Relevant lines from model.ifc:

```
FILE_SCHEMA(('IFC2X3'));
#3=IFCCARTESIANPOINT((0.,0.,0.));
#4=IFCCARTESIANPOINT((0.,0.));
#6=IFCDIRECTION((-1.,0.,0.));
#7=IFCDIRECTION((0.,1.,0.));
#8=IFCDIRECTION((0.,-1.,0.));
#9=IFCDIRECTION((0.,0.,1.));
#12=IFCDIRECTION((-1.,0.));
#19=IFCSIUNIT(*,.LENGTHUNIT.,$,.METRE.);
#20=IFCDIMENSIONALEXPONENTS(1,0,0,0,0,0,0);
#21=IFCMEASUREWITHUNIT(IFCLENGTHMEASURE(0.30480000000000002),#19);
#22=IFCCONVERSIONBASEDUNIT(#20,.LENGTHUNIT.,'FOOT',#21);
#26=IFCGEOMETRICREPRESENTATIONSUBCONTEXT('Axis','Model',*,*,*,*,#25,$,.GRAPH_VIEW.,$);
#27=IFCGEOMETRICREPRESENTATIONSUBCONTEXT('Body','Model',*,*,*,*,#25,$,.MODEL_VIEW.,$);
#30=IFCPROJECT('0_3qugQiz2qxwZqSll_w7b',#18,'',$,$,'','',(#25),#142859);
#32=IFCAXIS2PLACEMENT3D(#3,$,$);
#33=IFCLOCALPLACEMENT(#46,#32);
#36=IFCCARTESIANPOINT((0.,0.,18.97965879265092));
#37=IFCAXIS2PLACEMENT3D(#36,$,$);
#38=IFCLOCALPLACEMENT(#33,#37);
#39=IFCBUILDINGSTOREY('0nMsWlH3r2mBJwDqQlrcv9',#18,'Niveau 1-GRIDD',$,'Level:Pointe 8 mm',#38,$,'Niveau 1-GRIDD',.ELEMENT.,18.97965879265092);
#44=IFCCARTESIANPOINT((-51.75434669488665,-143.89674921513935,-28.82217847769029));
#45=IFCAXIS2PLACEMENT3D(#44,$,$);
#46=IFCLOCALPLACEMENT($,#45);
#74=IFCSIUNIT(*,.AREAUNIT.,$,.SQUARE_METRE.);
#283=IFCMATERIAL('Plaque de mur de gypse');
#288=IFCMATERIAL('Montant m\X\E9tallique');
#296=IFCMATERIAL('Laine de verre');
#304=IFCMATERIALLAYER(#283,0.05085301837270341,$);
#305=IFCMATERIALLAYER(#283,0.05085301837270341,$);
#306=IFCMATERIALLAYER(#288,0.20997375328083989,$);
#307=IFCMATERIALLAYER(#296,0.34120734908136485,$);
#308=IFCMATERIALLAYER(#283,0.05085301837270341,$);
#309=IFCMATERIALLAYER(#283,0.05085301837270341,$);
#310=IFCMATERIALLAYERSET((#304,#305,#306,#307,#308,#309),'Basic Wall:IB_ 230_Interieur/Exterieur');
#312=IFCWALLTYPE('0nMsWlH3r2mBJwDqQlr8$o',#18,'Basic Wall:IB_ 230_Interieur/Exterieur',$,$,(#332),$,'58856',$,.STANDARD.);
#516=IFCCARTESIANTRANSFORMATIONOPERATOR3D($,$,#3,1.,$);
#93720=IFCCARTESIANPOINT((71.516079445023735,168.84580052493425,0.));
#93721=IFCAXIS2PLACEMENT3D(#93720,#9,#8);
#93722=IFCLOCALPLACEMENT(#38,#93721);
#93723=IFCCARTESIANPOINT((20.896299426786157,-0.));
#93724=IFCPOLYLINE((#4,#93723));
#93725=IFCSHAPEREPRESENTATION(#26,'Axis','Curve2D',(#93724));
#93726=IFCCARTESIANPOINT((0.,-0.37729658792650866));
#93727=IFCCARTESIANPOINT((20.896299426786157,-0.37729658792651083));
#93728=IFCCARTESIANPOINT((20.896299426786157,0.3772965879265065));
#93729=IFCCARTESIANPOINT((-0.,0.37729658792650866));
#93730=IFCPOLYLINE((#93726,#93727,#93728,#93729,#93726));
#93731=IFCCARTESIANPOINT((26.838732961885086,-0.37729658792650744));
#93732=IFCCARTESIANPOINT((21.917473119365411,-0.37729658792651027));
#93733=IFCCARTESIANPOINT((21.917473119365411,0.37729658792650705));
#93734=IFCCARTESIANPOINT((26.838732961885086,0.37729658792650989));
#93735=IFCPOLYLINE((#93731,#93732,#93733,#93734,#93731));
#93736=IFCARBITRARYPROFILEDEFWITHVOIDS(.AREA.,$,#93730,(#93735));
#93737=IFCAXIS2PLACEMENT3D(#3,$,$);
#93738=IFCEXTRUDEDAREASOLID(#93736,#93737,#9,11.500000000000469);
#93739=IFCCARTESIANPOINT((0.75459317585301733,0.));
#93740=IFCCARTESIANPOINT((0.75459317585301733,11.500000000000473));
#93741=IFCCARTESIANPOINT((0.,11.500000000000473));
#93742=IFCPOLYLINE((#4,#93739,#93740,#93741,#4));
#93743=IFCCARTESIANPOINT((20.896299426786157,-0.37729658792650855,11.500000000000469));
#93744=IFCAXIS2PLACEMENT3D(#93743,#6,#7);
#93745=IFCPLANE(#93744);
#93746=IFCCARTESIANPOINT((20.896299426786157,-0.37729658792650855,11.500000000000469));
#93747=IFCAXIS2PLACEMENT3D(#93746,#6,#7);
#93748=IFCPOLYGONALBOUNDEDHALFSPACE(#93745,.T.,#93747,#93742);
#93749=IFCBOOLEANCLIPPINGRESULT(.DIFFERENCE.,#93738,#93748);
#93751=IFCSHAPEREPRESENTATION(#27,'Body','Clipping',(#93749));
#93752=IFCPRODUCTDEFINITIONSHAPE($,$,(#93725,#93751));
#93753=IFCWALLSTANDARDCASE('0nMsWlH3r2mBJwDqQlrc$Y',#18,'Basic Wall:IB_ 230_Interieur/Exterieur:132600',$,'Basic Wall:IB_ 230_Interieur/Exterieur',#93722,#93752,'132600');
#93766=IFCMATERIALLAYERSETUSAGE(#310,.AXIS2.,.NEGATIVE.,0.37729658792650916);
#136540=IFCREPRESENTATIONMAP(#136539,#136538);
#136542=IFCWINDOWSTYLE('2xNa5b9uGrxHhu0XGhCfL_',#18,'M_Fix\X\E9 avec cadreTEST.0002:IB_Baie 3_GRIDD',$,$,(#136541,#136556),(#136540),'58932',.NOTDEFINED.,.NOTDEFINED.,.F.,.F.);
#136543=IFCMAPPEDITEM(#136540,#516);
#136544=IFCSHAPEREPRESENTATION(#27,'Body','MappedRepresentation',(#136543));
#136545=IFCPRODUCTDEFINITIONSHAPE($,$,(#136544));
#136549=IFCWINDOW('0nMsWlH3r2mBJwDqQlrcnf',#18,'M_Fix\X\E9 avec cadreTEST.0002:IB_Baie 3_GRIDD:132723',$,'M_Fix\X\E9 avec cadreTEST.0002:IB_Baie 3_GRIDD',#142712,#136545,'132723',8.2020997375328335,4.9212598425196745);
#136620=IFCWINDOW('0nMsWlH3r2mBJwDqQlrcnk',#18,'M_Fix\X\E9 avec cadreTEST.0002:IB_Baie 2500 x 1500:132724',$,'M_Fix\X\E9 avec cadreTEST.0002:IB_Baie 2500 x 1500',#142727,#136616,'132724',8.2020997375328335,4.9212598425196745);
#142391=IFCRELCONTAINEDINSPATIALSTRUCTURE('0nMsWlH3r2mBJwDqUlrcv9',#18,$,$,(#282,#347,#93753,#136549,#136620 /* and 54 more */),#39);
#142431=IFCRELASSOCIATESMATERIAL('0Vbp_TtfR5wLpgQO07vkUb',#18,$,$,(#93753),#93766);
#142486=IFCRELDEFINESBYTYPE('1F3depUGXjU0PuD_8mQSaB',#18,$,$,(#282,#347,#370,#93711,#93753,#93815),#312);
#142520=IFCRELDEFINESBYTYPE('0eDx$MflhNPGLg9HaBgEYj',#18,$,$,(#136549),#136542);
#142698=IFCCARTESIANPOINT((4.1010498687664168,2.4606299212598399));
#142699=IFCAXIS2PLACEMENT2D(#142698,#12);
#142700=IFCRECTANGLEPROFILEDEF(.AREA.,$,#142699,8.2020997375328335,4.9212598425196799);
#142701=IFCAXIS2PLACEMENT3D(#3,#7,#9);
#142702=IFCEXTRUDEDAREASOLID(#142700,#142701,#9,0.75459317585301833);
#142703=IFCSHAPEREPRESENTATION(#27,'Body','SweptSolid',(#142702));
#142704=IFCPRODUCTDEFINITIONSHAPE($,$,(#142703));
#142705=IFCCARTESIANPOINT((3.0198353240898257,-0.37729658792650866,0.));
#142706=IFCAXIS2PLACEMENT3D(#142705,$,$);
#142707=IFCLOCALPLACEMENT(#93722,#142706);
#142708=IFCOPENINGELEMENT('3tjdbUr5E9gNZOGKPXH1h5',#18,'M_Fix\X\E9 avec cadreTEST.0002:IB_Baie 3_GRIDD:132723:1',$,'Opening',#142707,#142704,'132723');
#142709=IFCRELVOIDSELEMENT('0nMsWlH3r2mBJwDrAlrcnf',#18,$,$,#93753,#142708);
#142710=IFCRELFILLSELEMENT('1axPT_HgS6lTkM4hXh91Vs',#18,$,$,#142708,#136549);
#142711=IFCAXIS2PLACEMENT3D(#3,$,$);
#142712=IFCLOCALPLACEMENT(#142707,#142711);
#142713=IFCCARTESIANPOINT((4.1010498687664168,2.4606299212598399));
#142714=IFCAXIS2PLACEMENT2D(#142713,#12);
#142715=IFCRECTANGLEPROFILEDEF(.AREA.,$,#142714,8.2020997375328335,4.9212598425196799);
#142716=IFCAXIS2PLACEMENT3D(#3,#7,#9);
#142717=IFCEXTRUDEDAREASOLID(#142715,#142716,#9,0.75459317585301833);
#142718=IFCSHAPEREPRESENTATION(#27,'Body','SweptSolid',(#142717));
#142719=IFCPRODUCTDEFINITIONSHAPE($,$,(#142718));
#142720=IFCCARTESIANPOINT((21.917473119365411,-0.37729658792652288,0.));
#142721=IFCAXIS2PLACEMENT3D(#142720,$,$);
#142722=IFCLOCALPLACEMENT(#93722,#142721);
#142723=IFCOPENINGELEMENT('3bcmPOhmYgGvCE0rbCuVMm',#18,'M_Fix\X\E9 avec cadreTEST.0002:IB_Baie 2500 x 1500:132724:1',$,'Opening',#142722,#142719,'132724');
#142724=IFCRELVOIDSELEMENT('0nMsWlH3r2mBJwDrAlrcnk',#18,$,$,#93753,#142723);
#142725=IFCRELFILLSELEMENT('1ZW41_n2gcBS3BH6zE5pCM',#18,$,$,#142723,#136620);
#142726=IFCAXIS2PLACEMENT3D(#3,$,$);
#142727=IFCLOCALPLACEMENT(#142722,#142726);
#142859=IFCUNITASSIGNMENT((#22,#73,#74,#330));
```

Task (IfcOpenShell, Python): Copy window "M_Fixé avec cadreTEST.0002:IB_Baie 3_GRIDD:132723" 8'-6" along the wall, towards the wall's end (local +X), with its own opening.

```python
import ifcopenshell
import ifcopenshell.api.feature
import ifcopenshell.api.geometry
import ifcopenshell.api.root
import ifcopenshell.geom
import ifcopenshell.util.element
import ifcopenshell.util.placement
import ifcopenshell.util.shape
import ifcopenshell.util.unit

model = ifcopenshell.open("model.ifc")
unit_scale = ifcopenshell.util.unit.calculate_unit_scale(model)
settings = ifcopenshell.geom.settings()


def volume(element):
    """Net volume in cubic metres, openings subtracted."""
    shape = ifcopenshell.geom.create_shape(settings, element)
    return ifcopenshell.util.shape.get_volume(shape.geometry)


def reuse_history(source, copy):
    """copy_class also copies each property set's owner history, people and application; keep the originals."""
    for rel in copy.IsDefinedBy:
        if rel.is_a("IfcRelDefinesByProperties") and (history := rel.RelatingPropertyDefinition.OwnerHistory):
            rel.RelatingPropertyDefinition.OwnerHistory = source.OwnerHistory
            ifcopenshell.util.element.remove_deep2(model, history)


window = model.by_guid("0nMsWlH3r2mBJwDqQlrcnf")
opening = window.FillsVoids[0].RelatingOpeningElement
wall = opening.VoidsElements[0].RelatingBuildingElement
before = volume(wall)
shift = ifcopenshell.util.placement.get_local_placement(wall.ObjectPlacement)[:3, 0] * 102 * 0.0254 / unit_scale

# copy_class copies the void relationship, type, container and properties, but no geometry.
new_opening = ifcopenshell.api.root.copy_class(model, product=opening)
new_opening.Representation = ifcopenshell.util.element.copy_deep(
    model, opening.Representation, exclude=["IfcGeometricRepresentationContext", "IfcRepresentationMap"]
)
new_opening.Name = "M_Fixé avec cadreTEST.0002:IB_Baie 3_GRIDD"
new_opening.Tag = None
new_window = ifcopenshell.api.root.copy_class(model, product=window)
new_window.Representation = ifcopenshell.util.element.copy_deep(
    model, window.Representation, exclude=["IfcGeometricRepresentationContext", "IfcRepresentationMap"]
)
new_window.Name = "M_Fixé avec cadreTEST.0002:IB_Baie 3_GRIDD"
new_window.Tag = None
reuse_history(window, new_window)
fills = ifcopenshell.api.feature.add_filling(model, opening=new_opening, element=new_window)
fills.OwnerHistory = new_window.OwnerHistory  # required in IFC2X3

for old, new in ((opening, new_opening), (window, new_window)):
    matrix = ifcopenshell.util.placement.get_local_placement(old.ObjectPlacement)
    matrix[:3, 3] += shift
    ifcopenshell.api.geometry.edit_object_placement(model, product=new, matrix=matrix, is_si=False)

after = volume(wall)

print(f"wall volume {before:.3f} -> {after:.3f} m3")

model.write("model_edited.ifc")
```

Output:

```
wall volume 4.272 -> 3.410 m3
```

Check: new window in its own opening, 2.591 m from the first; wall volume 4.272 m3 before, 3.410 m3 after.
